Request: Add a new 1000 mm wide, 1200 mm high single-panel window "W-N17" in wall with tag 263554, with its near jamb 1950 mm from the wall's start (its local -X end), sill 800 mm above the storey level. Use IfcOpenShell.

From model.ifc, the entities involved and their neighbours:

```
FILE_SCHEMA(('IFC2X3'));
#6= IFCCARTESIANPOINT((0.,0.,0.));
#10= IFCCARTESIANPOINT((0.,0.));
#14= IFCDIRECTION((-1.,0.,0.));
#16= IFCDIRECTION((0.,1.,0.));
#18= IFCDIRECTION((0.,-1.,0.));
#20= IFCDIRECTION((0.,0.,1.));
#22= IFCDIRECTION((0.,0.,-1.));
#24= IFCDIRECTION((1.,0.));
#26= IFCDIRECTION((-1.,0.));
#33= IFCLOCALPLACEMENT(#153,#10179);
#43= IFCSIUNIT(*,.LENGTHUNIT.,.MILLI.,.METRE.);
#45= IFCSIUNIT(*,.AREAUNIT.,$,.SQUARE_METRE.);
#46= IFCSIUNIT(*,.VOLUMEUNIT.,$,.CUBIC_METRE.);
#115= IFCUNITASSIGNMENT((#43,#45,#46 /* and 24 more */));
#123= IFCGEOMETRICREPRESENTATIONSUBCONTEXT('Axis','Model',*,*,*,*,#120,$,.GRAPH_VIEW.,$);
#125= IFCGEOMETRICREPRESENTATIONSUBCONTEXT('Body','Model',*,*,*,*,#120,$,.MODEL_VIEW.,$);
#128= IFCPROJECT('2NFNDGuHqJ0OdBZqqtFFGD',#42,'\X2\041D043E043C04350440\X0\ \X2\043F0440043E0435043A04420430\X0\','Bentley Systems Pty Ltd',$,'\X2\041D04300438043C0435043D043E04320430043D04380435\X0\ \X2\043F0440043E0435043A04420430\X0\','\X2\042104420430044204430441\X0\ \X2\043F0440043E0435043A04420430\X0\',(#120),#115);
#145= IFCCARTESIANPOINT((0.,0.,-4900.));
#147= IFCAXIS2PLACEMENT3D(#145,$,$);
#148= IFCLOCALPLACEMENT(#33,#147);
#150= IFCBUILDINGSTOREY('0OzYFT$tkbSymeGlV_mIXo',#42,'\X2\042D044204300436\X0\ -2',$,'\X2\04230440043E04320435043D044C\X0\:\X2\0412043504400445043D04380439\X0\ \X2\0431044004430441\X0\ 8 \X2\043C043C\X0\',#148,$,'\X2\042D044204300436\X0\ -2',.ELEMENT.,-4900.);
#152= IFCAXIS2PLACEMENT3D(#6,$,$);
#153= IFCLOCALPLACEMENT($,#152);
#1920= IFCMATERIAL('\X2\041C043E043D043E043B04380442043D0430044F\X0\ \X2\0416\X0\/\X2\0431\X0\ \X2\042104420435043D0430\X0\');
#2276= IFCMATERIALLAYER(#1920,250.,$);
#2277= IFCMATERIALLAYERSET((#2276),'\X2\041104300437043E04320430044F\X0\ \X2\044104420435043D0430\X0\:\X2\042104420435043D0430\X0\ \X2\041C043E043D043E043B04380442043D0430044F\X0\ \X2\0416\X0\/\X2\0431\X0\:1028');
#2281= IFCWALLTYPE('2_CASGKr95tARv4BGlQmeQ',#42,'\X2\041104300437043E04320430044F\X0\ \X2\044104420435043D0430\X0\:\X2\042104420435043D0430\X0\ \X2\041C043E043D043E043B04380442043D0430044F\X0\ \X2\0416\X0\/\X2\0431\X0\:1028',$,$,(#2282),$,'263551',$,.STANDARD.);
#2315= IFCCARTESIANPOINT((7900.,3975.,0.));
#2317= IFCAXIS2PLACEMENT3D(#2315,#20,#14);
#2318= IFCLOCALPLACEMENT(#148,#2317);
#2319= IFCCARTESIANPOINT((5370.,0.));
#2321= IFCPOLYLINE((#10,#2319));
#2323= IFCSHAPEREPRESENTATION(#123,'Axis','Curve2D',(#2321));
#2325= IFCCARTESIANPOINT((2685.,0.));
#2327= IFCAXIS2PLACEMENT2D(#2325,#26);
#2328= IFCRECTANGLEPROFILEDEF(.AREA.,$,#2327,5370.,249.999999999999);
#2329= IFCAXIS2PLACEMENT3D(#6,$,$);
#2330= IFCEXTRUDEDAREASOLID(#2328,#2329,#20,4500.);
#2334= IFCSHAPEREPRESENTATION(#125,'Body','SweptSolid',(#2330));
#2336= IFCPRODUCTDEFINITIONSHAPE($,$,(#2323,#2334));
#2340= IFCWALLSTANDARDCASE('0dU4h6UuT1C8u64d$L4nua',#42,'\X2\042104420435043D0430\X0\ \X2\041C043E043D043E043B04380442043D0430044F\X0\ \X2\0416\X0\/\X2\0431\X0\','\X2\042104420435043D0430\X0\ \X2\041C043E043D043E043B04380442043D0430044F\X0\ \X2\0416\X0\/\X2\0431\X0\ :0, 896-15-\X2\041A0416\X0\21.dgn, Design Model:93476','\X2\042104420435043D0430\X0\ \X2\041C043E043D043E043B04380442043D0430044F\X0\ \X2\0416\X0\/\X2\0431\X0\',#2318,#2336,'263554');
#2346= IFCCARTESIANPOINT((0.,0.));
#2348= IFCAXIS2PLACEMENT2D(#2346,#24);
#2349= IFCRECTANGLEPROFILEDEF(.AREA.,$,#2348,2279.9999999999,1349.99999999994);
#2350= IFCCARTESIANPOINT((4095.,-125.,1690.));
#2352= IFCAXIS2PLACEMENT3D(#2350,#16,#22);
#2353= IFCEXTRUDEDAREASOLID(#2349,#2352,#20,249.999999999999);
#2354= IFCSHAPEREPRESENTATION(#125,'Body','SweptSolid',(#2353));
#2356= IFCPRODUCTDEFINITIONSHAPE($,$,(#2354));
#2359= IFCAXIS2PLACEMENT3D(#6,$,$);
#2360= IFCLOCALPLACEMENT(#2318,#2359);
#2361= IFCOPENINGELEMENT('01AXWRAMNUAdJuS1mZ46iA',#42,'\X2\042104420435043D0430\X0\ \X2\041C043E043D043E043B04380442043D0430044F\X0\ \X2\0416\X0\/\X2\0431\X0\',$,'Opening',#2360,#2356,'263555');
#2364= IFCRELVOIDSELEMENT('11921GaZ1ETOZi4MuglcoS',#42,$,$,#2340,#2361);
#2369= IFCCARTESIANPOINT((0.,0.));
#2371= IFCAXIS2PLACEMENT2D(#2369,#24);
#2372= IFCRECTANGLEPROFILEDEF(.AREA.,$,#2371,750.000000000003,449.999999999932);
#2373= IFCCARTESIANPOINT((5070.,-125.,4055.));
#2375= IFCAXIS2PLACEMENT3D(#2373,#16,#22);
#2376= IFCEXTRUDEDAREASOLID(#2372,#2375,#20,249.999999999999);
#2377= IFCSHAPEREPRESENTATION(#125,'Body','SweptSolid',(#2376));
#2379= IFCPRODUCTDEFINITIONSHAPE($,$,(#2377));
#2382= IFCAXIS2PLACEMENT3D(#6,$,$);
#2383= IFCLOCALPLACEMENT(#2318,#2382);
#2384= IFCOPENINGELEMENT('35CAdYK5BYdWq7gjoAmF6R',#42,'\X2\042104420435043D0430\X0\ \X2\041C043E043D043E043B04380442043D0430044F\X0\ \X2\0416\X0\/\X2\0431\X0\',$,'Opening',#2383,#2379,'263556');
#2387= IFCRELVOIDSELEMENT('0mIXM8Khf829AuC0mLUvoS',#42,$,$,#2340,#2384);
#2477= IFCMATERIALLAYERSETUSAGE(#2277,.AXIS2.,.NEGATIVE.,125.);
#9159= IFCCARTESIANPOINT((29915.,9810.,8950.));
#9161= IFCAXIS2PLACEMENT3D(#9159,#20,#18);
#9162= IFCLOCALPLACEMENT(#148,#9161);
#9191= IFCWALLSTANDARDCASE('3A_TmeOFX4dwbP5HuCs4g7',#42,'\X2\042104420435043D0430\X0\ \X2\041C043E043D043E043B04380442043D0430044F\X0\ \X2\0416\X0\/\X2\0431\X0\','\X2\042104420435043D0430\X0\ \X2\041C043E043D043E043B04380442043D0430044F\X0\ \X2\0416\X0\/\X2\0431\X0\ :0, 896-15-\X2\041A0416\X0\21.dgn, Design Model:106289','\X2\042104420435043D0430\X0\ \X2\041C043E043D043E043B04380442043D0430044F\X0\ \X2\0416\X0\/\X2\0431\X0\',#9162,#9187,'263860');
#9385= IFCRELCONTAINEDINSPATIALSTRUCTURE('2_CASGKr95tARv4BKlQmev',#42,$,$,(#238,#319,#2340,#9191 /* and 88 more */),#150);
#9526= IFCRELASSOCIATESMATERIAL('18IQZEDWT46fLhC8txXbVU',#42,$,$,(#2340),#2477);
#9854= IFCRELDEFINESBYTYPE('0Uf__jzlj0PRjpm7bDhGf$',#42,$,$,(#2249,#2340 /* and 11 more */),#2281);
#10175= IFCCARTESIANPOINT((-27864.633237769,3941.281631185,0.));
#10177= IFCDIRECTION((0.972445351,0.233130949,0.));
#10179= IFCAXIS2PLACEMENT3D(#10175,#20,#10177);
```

```python
import numpy as np
import ifcopenshell
import ifcopenshell.api.feature
import ifcopenshell.api.geometry
import ifcopenshell.api.root
import ifcopenshell.api.spatial
import ifcopenshell.api.type
import ifcopenshell.geom
import ifcopenshell.util.element
import ifcopenshell.util.placement
import ifcopenshell.util.representation
import ifcopenshell.util.shape
import ifcopenshell.util.unit

model = ifcopenshell.open("model.ifc")
unit_scale = ifcopenshell.util.unit.calculate_unit_scale(model)
settings = ifcopenshell.geom.settings()


def volume(element):
    """Net volume in cubic metres, openings subtracted."""
    shape = ifcopenshell.geom.create_shape(settings, element)
    return ifcopenshell.util.shape.get_volume(shape.geometry)


wall = model.by_guid("0dU4h6UuT1C8u64d$L4nua")
storey = ifcopenshell.util.element.get_container(wall, ifc_class="IfcBuildingStorey")
context = ifcopenshell.util.representation.get_context(model, "Model", "Body", "MODEL_VIEW")
before = volume(wall)

width, height, from_end, sill = 1, 1.2, 1.95, 0.8  # metres

# The wall runs along its own X axis, and the end named is its -X end.
wall_shape = ifcopenshell.geom.create_shape(settings, wall)
x, y, z = ifcopenshell.util.shape.get_vertices(wall_shape.geometry).T
start = x.min() + from_end
face, thickness = float(y.min()), float(y.max() - y.min())
wall_matrix = ifcopenshell.util.placement.get_local_placement(wall.ObjectPlacement)
level = ifcopenshell.util.placement.get_local_placement(storey.ObjectPlacement)[2, 3]


def in_wall(x, y):
    """Placement at x, y metres in the wall's axes, at sill height."""
    matrix = wall_matrix.copy()
    matrix[:, 3] = wall_matrix @ np.array([x / unit_scale, y / unit_scale, 0.0, 1.0])
    matrix[2, 3] = level + sill / unit_scale
    return matrix


# Opening: a box that overshoots both wall faces by 50 mm.
opening = ifcopenshell.api.root.create_entity(model, ifc_class="IfcOpeningElement")
box = ifcopenshell.api.geometry.add_wall_representation(
    model, context=context, length=width, height=height, thickness=thickness + 0.1
)
ifcopenshell.api.geometry.assign_representation(model, product=opening, representation=box)
ifcopenshell.api.geometry.edit_object_placement(model, product=opening, matrix=in_wall(start, face - 0.05), is_si=False)
ifcopenshell.api.feature.add_feature(model, feature=opening, element=wall)

window = ifcopenshell.api.root.create_entity(model, ifc_class="IfcWindow", name="W-N17")
window.OverallWidth, window.OverallHeight = width / unit_scale, height / unit_scale
body = ifcopenshell.api.geometry.add_window_representation(
    model,
    context=context,
    overall_width=window.OverallWidth,
    overall_height=window.OverallHeight,
    partition_type="SINGLE_PANEL",
)
ifcopenshell.api.geometry.assign_representation(model, product=window, representation=body)
ifcopenshell.api.spatial.assign_container(model, products=[window], relating_structure=storey)
fills = ifcopenshell.api.feature.add_filling(model, opening=opening, element=window)
fills.OwnerHistory = window.OwnerHistory  # required in IFC2X3

# IFC2X3 keeps the operation on the window style.
style = ifcopenshell.api.root.create_entity(model, ifc_class="IfcWindowStyle", name="W-N17")
style.OperationType, style.ConstructionType = "SINGLE_PANEL", "NOTDEFINED"
style.ParameterTakesPrecedence = style.Sizeable = False
ifcopenshell.api.type.assign_type(model, related_objects=[window], relating_type=style)

# Centre the window in the wall's thickness.
ifcopenshell.api.geometry.edit_object_placement(model, product=window, matrix=in_wall(start, face), is_si=False)
window_shape = ifcopenshell.geom.create_shape(settings, window)
depth = ifcopenshell.util.shape.get_vertices(window_shape.geometry)[:, 1]
offset = face + thickness / 2 - (depth.min() + depth.max()) / 2
ifcopenshell.api.geometry.edit_object_placement(model, product=window, matrix=in_wall(start, offset), is_si=False)

after = volume(wall)

print(f"wall volume {before:.3f} -> {after:.3f} m3")

model.write("model_updated.ifc")
```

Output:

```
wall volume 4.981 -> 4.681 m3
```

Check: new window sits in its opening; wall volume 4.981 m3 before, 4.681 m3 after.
